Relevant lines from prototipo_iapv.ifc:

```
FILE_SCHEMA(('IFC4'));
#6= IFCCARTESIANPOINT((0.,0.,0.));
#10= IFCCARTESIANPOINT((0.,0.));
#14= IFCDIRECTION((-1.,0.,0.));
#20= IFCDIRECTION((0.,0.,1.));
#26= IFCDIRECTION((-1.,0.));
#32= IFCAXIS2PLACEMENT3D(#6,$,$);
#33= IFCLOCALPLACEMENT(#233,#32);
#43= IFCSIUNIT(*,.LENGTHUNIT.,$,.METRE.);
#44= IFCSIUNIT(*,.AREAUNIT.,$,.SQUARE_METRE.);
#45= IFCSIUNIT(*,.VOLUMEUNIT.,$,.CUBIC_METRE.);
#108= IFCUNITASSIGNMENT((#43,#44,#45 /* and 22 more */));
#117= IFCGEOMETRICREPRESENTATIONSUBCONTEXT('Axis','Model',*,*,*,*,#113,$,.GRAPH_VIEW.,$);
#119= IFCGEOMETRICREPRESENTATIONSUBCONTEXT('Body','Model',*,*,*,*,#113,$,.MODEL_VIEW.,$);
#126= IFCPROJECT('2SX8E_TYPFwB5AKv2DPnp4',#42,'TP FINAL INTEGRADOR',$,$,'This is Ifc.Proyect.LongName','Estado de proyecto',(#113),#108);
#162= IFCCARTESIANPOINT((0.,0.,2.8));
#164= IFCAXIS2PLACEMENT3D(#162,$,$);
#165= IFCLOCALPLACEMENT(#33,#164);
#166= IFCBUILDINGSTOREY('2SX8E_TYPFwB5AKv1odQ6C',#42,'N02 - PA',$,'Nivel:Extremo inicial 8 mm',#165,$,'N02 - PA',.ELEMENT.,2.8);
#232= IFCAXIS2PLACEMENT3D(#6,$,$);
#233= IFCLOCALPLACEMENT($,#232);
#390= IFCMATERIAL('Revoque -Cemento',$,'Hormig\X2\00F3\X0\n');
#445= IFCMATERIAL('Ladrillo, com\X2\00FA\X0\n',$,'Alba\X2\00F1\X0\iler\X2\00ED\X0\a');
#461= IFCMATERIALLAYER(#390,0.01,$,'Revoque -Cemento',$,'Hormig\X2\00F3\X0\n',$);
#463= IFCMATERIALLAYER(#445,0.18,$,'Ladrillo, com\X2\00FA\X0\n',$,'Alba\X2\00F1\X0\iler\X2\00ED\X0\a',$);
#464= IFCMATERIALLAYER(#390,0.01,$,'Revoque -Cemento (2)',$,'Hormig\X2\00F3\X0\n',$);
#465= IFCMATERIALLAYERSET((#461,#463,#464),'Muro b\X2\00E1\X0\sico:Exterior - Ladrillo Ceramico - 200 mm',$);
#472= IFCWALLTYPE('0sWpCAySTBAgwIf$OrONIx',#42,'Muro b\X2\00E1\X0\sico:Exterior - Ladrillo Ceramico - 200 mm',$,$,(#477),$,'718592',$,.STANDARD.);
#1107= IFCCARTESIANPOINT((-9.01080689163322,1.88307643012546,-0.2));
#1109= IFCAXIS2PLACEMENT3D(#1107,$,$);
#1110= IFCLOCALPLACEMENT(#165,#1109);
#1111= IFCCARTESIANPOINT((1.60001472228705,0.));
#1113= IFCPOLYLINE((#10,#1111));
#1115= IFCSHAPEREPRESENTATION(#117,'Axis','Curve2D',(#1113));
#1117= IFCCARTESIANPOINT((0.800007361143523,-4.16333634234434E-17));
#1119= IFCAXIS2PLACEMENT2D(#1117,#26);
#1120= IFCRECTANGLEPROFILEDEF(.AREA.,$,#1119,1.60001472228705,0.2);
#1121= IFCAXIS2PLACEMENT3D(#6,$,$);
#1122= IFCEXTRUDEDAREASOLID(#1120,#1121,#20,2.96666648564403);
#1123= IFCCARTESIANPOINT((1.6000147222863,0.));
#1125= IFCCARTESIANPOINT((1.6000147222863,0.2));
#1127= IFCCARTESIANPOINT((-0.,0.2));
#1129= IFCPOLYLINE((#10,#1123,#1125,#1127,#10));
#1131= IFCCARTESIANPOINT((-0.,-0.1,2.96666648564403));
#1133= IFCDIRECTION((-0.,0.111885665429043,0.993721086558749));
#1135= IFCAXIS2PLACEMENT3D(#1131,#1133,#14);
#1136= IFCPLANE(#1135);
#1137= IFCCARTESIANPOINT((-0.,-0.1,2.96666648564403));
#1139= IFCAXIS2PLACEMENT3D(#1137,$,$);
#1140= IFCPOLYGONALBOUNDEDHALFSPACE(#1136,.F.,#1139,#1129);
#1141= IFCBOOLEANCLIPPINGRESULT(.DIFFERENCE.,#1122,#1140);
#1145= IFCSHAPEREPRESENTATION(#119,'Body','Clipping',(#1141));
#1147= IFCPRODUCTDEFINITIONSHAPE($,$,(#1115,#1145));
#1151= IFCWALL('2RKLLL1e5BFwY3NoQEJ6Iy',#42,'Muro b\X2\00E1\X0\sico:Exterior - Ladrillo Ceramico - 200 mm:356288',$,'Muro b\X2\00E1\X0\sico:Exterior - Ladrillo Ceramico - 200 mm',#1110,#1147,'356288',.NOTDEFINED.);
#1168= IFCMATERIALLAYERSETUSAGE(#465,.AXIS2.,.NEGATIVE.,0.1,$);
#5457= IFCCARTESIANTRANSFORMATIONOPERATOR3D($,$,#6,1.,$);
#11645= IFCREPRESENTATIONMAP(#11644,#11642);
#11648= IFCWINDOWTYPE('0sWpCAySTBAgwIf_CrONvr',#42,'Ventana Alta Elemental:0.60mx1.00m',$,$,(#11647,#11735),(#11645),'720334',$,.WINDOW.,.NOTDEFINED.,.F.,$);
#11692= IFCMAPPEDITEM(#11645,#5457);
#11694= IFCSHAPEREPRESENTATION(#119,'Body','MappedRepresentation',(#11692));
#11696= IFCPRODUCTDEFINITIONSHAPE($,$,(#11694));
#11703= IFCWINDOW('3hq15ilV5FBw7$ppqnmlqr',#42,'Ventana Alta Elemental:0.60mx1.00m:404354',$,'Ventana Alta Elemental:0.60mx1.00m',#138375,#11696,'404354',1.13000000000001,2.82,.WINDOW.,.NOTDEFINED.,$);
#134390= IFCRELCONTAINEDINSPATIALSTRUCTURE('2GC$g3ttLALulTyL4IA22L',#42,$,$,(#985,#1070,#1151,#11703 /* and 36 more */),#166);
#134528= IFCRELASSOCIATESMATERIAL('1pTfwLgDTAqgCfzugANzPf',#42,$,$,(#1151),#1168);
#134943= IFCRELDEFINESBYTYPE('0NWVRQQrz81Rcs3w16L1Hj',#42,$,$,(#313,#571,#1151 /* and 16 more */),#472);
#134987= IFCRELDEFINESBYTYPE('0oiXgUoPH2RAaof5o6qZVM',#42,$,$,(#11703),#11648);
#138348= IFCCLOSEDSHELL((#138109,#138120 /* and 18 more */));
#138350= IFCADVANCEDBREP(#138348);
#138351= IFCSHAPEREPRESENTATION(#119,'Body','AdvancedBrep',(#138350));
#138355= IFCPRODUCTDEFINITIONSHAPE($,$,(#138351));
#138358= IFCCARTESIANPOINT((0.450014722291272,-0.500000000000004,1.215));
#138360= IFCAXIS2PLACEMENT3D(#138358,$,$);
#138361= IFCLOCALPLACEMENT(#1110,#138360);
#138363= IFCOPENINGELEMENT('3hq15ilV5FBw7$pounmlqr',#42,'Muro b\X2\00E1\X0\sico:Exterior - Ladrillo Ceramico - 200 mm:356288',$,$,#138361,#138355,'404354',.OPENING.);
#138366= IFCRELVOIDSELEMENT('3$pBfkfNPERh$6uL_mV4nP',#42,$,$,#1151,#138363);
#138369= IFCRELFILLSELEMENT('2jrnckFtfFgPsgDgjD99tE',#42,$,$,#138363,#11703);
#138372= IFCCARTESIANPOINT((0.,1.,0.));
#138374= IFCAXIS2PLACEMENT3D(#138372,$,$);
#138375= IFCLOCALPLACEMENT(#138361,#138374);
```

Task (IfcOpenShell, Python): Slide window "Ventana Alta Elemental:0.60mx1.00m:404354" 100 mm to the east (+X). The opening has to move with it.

```python
import ifcopenshell
import ifcopenshell.api.geometry
import ifcopenshell.util.placement

model = ifcopenshell.open("prototipo_iapv.ifc")

window = model.by_guid("3hq15ilV5FBw7$ppqnmlqr")
opening = window.FillsVoids[0].RelatingOpeningElement
wall = opening.VoidsElements[0].RelatingBuildingElement

wall_matrix = ifcopenshell.util.placement.get_local_placement(wall.ObjectPlacement)
shift = wall_matrix[:3, 0] * 0.1
before = ifcopenshell.util.placement.get_local_placement(window.ObjectPlacement)[:3, 3].copy()

# The window is placed relative to its opening, so it follows when the opening moves.
matrix = ifcopenshell.util.placement.get_local_placement(opening.ObjectPlacement)
matrix[:3, 3] += shift
ifcopenshell.api.geometry.edit_object_placement(
    model, product=opening, matrix=matrix, is_si=False, should_transform_children=True
)

after = ifcopenshell.util.placement.get_local_placement(window.ObjectPlacement)[:3, 3]
print("window moved by", (after - before).round(3) + 0.0)

model.write("prototipo_iapv-out.ifc")
```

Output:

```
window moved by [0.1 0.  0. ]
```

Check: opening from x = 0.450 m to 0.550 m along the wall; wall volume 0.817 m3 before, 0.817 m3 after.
